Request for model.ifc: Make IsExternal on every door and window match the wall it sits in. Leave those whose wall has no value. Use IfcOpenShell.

First a look at what the model holds.

```python
import ifcopenshell
import ifcopenshell.util.element

model = ifcopenshell.open("model.ifc")
print(model.schema)
seen = {}
for e in model.by_type("IfcDoor") + model.by_type("IfcWindow"):
    if not e.FillsVoids:
        continue
    host = e.FillsVoids[0].RelatingOpeningElement.VoidsElements[0].RelatingBuildingElement
    own = ifcopenshell.util.element.get_pset(e, f"Pset_{e.is_a()[3:].removesuffix('StandardCase')}Common", "IsExternal")
    wall = ifcopenshell.util.element.get_pset(host, "Pset_WallCommon", "IsExternal")
    seen[e.is_a(), own, wall] = seen.get((e.is_a(), own, wall), 0) + 1
for (cls, own, wall), count in sorted(seen.items(), key=str):
    print(count, cls, "IsExternal:", own, "| host wall:", wall)
```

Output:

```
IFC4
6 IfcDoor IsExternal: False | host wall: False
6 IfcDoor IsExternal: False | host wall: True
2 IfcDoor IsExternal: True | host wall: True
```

```python
import ifcopenshell
import ifcopenshell.api.pset
import ifcopenshell.util.element

model = ifcopenshell.open("model.ifc")

count = 0
for ifc_class, pset_name in (("IfcDoor", "Pset_DoorCommon"), ("IfcWindow", "Pset_WindowCommon")):
    for e in model.by_type(ifc_class):
        if not e.FillsVoids:
            continue
        host = e.FillsVoids[0].RelatingOpeningElement.VoidsElements[0].RelatingBuildingElement
        external = ifcopenshell.util.element.get_pset(host, "Pset_WallCommon", "IsExternal")
        if external is None or ifcopenshell.util.element.get_pset(e, pset_name, "IsExternal") == external:
            continue
        pset = ifcopenshell.api.pset.add_pset(model, product=e, name=pset_name)
        ifcopenshell.api.pset.edit_pset(model, pset=pset, properties={"IsExternal": external})
        count += 1

print(count, "updated")

model.write("model_updated.ifc")
```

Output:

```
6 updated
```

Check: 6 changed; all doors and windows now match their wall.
